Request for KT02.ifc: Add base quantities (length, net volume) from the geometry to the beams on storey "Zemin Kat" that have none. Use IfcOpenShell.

First a look at what the model holds.

```python
import ifcopenshell
import ifcopenshell.util.element
import ifcopenshell.util.unit

model = ifcopenshell.open("KT02.ifc")
print(model.schema)
for unit_type in ("LENGTHUNIT", "AREAUNIT", "VOLUMEUNIT"):
    print(unit_type, ifcopenshell.util.unit.calculate_unit_scale(model, unit_type))
storey = next(s for s in model.by_type("IfcBuildingStorey") if s.Name == "Zemin Kat")
beams = [e for e in ifcopenshell.util.element.get_decomposition(storey) if e.is_a("IfcBeam")]
for e in sorted(beams, key=lambda e: e.id()):
    print(e.id(), e.is_a(), e.Name, list(ifcopenshell.util.element.get_psets(e, qtos_only=True)), sep=" | ")
```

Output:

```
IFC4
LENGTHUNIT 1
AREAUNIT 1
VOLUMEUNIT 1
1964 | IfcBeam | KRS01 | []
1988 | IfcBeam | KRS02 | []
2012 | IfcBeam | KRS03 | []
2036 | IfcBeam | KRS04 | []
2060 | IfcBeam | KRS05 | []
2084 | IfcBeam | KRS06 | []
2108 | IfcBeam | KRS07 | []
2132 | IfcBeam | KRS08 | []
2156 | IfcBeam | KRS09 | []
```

```python
import ifcopenshell
import ifcopenshell.api.pset
import ifcopenshell.geom
import ifcopenshell.util.element
import ifcopenshell.util.shape
import ifcopenshell.util.unit

model = ifcopenshell.open("KT02.ifc")
unit_scale = ifcopenshell.util.unit.calculate_unit_scale(model)
volume_scale = ifcopenshell.util.unit.calculate_unit_scale(model, "VOLUMEUNIT")
settings = ifcopenshell.geom.settings()

storey = next(s for s in model.by_type("IfcBuildingStorey") if s.Name == "Zemin Kat")
beams = [e for e in ifcopenshell.util.element.get_decomposition(storey) if e.is_a("IfcBeam")]

for e in sorted(beams, key=lambda e: e.id()):
    if ifcopenshell.util.element.get_psets(e, qtos_only=True, should_inherit=False):
        continue
    # Geometry comes back in metres, in the element's own axes.
    shape = ifcopenshell.geom.create_shape(settings, e)
    values = {
        "Length": ifcopenshell.util.shape.get_max_xyz(shape.geometry) / unit_scale,
        "NetVolume": ifcopenshell.util.shape.get_volume(shape.geometry) / volume_scale,
    }
    qto = ifcopenshell.api.pset.add_qto(model, product=e, name="Qto_BeamBaseQuantities")
    ifcopenshell.api.pset.edit_qto(model, qto=qto, properties=values)
    print(e.id(), {k: round(v, 3) for k, v in values.items()})

model.write("KT02_rev.ifc")
```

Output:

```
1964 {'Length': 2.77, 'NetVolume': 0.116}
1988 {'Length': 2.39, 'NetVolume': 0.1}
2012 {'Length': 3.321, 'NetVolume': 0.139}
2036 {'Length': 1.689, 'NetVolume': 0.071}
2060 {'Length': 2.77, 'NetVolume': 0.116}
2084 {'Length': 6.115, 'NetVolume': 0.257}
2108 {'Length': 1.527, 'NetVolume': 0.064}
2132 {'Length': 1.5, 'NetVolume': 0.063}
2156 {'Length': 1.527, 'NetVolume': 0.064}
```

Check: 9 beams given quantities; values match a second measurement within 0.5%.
